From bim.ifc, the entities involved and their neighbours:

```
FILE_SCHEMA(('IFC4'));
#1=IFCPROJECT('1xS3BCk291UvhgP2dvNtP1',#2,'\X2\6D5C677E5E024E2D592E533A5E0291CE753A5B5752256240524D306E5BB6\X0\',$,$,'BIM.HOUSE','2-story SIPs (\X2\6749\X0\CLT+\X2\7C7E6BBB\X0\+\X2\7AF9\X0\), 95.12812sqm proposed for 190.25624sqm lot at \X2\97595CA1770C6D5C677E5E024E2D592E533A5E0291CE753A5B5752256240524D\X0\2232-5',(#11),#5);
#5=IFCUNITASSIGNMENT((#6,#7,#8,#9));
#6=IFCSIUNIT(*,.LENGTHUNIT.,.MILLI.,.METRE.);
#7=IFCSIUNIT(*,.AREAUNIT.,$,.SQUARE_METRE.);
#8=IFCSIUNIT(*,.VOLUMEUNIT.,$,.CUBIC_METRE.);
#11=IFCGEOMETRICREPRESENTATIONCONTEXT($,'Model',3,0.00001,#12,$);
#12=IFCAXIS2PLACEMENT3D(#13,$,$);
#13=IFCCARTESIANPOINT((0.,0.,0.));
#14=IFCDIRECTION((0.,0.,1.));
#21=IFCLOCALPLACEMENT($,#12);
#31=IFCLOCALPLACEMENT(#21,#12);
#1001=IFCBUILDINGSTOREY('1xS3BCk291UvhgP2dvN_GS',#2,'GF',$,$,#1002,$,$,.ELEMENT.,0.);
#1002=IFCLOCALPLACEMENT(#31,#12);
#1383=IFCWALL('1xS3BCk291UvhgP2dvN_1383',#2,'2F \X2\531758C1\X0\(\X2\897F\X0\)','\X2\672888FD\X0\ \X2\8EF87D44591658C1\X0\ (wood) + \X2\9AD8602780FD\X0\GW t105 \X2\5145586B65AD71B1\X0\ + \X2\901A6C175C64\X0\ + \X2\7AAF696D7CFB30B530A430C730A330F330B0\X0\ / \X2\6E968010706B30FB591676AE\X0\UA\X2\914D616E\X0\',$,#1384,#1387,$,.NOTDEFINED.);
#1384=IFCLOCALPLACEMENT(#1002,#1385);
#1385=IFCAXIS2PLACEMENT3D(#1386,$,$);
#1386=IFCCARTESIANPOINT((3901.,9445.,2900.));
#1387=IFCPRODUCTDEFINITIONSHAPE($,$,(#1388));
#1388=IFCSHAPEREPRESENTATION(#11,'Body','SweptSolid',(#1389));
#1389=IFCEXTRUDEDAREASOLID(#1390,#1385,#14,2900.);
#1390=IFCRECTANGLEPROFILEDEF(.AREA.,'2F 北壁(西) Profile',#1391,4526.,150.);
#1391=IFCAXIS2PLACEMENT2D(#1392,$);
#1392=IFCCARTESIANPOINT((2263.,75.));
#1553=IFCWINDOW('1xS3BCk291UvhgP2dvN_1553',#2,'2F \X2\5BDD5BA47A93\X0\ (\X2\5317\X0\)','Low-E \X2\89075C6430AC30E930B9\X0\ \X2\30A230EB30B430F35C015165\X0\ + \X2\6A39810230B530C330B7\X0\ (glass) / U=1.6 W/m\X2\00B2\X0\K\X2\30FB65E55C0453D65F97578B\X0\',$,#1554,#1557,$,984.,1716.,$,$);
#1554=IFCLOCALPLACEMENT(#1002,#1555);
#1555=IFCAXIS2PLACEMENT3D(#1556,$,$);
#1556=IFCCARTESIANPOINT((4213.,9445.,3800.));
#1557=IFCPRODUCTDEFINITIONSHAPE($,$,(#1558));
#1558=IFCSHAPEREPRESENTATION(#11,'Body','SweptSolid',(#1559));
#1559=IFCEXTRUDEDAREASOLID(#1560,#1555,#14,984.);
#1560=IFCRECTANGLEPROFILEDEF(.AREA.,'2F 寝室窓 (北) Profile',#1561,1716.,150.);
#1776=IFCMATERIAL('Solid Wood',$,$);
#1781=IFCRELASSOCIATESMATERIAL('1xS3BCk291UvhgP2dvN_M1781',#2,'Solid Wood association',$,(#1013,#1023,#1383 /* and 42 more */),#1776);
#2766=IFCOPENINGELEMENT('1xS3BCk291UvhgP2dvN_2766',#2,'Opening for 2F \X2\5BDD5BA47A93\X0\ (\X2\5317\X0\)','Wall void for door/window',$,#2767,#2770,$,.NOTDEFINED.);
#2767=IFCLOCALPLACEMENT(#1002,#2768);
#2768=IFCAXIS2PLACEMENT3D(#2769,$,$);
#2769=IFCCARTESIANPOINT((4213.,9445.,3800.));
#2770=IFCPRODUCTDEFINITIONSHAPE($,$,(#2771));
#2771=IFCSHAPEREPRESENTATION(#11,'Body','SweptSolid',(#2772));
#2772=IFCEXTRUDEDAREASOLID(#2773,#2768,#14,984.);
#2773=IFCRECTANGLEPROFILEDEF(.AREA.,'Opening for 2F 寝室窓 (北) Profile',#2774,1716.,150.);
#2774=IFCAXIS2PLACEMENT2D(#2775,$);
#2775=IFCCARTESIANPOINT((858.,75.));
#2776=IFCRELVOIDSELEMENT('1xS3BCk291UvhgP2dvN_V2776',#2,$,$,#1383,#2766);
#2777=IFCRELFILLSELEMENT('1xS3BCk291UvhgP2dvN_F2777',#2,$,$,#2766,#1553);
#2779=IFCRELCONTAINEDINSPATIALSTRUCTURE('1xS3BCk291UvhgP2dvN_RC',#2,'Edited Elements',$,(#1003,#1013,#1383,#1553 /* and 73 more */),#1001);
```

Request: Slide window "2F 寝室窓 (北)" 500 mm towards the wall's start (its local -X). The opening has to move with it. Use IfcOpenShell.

```python
import ifcopenshell
import ifcopenshell.api.geometry
import ifcopenshell.util.placement
import ifcopenshell.util.unit

model = ifcopenshell.open("bim.ifc")
unit_scale = ifcopenshell.util.unit.calculate_unit_scale(model)

window = model.by_guid("1xS3BCk291UvhgP2dvN_1553")
opening = window.FillsVoids[0].RelatingOpeningElement
wall = opening.VoidsElements[0].RelatingBuildingElement

wall_matrix = ifcopenshell.util.placement.get_local_placement(wall.ObjectPlacement)
shift = wall_matrix[:3, 0] * -0.5 / unit_scale
before = ifcopenshell.util.placement.get_local_placement(window.ObjectPlacement)[:3, 3].copy()

# The window is not placed relative to its opening, so move both.
for product in (opening, window):
    matrix = ifcopenshell.util.placement.get_local_placement(product.ObjectPlacement)
    matrix[:3, 3] += shift
    ifcopenshell.api.geometry.edit_object_placement(model, product=product, matrix=matrix, is_si=False)

after = ifcopenshell.util.placement.get_local_placement(window.ObjectPlacement)[:3, 3]
print("window moved by", (after - before).round(3) + 0.0)

model.write("bim_updated.ifc")
```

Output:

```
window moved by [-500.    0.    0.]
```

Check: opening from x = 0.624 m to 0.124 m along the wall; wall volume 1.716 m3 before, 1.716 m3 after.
